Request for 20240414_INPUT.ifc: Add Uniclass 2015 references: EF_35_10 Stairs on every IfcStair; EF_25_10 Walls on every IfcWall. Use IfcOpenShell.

First a look at what the model holds.

```python
import ifcopenshell

model = ifcopenshell.open("20240414_INPUT.ifc")
print(model.schema)
print("classifications:", [c.Name for c in model.by_type("IfcClassification")])
for ifc_class in ("IfcDoor", "IfcRoof", "IfcStair", "IfcWall", "IfcWindow"):
    print(ifc_class, len(model.by_type(ifc_class)))
```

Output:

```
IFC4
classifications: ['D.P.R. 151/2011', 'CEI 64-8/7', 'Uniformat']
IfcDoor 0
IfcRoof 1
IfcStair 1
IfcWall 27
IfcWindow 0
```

```python
import ifcopenshell
import ifcopenshell.api.classification

model = ifcopenshell.open("20240414_INPUT.ifc")

system = ifcopenshell.api.classification.add_classification(model, classification="Uniclass 2015")

codes = {
    "IfcStair": ("EF_35_10", "Stairs"),
    "IfcWall": ("EF_25_10", "Walls"),
}
for ifc_class, (code, name) in codes.items():
    products = model.by_type(ifc_class)
    ifcopenshell.api.classification.add_reference(
        model, products=products, classification=system, identification=code, name=name
    )
    print(code, len(products))

model.write("20240414_INPUT_edited.ifc")
```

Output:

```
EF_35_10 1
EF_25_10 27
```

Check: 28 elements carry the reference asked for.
